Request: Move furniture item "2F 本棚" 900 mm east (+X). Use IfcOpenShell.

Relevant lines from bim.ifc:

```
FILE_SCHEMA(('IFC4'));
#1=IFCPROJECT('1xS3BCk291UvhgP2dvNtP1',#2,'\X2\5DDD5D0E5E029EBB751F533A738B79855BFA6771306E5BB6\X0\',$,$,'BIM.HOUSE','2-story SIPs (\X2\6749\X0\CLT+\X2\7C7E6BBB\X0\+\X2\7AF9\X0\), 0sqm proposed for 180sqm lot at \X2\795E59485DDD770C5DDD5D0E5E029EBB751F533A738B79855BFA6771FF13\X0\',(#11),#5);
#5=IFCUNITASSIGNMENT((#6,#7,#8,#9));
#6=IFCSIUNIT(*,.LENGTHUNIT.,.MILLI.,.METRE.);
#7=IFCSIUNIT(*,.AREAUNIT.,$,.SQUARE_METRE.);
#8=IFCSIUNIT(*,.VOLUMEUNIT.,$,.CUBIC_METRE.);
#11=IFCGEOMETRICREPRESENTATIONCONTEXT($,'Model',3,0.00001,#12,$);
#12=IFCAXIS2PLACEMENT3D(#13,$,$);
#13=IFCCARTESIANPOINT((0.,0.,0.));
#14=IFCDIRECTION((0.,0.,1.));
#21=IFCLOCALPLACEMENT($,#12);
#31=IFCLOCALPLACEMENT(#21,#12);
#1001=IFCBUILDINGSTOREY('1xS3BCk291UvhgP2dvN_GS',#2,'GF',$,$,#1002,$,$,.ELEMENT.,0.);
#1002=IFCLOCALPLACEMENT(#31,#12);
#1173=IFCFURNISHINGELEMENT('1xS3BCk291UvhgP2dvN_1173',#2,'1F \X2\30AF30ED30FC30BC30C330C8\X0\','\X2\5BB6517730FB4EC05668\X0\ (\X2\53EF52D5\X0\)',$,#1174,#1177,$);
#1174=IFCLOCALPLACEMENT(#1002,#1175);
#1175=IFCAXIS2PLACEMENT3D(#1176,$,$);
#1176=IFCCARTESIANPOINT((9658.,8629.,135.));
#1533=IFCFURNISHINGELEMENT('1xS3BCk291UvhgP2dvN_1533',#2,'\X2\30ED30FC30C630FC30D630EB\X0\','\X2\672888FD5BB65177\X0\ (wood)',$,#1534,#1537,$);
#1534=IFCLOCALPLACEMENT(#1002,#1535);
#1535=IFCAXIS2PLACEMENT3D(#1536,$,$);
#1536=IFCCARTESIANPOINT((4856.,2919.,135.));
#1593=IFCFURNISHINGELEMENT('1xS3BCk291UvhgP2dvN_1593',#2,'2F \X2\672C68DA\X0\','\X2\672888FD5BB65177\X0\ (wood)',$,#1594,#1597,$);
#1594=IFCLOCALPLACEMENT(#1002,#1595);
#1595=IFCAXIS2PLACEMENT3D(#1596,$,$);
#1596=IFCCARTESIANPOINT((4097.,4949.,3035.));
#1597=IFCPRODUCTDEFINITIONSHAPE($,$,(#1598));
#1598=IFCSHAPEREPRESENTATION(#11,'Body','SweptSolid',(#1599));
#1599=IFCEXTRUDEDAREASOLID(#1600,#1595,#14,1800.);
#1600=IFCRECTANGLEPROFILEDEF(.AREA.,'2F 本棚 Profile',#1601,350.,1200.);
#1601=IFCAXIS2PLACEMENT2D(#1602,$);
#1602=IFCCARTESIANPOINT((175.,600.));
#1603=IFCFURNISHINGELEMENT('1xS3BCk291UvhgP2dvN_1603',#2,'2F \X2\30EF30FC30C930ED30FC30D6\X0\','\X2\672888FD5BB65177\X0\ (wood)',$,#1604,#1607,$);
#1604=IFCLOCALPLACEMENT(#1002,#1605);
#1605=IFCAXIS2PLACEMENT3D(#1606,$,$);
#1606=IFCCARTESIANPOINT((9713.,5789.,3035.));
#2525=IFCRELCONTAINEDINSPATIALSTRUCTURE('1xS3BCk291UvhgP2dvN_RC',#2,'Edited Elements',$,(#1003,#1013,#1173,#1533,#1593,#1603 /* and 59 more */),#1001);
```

```python
import ifcopenshell
import ifcopenshell.api.geometry
import ifcopenshell.util.placement

model = ifcopenshell.open("bim.ifc")

item = model.by_guid("1xS3BCk291UvhgP2dvN_1593")
matrix = ifcopenshell.util.placement.get_local_placement(item.ObjectPlacement)
matrix[0, 3] += 900.0
ifcopenshell.api.geometry.edit_object_placement(model, product=item, matrix=matrix, is_si=False)

print(ifcopenshell.util.placement.get_local_placement(item.ObjectPlacement).round(3) + 0.0)

model.write("bim_updated.ifc")
```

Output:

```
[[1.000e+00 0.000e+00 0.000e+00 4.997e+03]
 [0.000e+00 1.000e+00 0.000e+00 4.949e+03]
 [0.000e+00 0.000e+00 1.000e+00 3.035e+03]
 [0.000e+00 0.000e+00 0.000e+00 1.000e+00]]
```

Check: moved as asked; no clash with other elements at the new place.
